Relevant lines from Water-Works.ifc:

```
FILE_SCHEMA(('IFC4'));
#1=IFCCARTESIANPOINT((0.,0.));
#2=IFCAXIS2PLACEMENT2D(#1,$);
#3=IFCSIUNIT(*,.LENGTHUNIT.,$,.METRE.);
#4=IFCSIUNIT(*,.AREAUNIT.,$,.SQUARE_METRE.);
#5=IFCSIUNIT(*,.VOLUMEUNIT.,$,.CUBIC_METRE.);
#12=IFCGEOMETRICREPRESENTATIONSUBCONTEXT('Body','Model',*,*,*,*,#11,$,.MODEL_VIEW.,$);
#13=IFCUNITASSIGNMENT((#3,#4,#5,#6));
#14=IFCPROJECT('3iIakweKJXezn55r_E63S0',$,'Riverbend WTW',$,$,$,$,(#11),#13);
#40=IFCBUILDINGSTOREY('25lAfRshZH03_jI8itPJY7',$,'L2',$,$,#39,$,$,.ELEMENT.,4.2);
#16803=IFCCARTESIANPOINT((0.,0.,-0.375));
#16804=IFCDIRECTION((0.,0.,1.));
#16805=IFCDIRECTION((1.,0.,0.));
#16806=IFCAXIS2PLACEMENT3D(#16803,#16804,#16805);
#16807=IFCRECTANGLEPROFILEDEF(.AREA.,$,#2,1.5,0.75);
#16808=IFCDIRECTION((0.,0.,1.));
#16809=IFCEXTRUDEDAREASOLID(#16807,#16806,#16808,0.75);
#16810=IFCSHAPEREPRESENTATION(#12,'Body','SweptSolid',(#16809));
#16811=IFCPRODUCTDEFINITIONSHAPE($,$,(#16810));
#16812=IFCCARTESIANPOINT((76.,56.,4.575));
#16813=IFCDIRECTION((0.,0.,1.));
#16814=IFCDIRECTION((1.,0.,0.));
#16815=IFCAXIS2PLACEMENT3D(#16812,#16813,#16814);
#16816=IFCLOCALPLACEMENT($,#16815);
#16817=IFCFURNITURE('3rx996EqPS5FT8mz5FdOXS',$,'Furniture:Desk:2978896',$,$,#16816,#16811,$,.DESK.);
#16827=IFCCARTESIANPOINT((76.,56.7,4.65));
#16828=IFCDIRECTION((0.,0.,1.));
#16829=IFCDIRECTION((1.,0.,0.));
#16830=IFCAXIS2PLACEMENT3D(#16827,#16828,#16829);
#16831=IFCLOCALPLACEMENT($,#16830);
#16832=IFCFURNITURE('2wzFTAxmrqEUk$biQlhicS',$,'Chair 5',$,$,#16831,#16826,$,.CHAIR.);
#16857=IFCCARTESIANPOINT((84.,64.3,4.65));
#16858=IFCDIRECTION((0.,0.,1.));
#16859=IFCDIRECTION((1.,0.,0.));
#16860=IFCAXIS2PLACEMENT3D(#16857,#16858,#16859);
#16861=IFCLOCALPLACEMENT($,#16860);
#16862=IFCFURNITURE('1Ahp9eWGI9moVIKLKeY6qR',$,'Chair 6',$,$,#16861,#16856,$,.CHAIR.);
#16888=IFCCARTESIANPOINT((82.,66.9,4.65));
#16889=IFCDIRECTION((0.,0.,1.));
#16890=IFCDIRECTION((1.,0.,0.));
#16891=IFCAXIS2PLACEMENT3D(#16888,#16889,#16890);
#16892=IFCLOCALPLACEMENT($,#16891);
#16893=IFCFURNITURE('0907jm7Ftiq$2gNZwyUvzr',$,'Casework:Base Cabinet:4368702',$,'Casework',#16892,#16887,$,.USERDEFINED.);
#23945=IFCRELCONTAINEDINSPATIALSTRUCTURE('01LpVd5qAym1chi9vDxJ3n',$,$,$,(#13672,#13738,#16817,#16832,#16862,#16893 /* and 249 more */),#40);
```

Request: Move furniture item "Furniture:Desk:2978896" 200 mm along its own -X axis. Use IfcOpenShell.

```python
import ifcopenshell
import ifcopenshell.api.geometry
import ifcopenshell.util.placement
import ifcopenshell.util.unit

model = ifcopenshell.open("Water-Works.ifc")
unit_scale = ifcopenshell.util.unit.calculate_unit_scale(model)

item = model.by_guid("3rx996EqPS5FT8mz5FdOXS")
matrix = ifcopenshell.util.placement.get_local_placement(item.ObjectPlacement)
matrix[:3, 3] -= matrix[:3, 0] * 0.2 / unit_scale
ifcopenshell.api.geometry.edit_object_placement(model, product=item, matrix=matrix, is_si=False)

print(ifcopenshell.util.placement.get_local_placement(item.ObjectPlacement).round(3) + 0.0)

model.write("Water-Works_edited.ifc")
```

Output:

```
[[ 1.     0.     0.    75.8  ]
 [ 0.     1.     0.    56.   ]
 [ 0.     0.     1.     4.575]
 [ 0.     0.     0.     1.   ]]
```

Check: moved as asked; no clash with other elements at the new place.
